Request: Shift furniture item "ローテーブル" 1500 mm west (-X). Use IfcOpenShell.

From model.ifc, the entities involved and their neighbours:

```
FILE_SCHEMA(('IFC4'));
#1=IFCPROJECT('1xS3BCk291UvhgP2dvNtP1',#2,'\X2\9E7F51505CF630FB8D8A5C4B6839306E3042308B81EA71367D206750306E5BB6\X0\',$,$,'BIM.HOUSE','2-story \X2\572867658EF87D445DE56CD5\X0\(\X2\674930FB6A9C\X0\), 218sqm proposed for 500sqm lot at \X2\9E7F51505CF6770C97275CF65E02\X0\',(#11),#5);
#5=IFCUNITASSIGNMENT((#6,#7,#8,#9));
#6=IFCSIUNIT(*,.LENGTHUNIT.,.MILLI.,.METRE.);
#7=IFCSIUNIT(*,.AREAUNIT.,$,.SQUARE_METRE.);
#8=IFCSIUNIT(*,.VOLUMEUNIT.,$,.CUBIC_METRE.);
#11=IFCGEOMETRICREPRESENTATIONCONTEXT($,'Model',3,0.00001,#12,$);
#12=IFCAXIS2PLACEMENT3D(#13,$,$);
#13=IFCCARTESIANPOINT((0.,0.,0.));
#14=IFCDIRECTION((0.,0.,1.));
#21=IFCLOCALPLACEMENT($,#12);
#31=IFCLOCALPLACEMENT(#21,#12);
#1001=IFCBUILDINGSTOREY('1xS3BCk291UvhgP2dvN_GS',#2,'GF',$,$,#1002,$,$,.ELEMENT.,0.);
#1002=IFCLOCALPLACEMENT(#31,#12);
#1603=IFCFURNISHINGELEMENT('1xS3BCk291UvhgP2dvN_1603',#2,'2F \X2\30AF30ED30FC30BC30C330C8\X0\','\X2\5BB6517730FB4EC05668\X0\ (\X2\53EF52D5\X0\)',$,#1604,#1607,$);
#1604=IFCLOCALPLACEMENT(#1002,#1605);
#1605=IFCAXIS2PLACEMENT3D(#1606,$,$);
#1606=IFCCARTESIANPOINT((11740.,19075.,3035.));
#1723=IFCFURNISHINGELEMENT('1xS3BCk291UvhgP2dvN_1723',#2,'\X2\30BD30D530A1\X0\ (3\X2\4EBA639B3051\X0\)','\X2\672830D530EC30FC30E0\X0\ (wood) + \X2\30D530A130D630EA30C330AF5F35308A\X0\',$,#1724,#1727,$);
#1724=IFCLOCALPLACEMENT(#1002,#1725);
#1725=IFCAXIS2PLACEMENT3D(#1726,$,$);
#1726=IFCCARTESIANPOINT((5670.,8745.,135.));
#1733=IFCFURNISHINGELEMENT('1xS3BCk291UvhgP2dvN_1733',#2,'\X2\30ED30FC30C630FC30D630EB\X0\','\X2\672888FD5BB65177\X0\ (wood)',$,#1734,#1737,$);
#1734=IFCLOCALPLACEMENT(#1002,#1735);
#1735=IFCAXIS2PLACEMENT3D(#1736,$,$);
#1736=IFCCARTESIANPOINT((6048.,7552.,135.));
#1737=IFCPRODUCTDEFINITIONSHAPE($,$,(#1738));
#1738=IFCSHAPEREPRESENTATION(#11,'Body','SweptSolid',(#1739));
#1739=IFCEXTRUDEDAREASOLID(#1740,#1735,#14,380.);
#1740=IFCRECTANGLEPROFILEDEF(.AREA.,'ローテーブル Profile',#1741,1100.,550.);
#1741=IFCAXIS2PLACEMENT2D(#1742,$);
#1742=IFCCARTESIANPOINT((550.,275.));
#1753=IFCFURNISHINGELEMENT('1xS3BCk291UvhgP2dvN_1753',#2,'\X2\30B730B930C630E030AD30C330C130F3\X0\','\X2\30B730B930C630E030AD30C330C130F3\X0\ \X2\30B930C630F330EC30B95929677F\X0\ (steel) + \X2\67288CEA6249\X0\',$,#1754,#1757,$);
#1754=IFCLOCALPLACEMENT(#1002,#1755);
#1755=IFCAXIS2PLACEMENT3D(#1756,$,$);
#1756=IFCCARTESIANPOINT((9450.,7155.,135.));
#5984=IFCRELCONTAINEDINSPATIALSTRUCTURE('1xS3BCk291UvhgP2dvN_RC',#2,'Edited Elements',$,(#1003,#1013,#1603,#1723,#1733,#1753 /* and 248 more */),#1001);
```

```python
import ifcopenshell
import ifcopenshell.api.geometry
import ifcopenshell.util.placement

model = ifcopenshell.open("model.ifc")

item = model.by_guid("1xS3BCk291UvhgP2dvN_1733")
matrix = ifcopenshell.util.placement.get_local_placement(item.ObjectPlacement)
matrix[0, 3] -= 1500.0
ifcopenshell.api.geometry.edit_object_placement(model, product=item, matrix=matrix, is_si=False)

print(ifcopenshell.util.placement.get_local_placement(item.ObjectPlacement).round(3) + 0.0)

model.write("model_updated.ifc")
```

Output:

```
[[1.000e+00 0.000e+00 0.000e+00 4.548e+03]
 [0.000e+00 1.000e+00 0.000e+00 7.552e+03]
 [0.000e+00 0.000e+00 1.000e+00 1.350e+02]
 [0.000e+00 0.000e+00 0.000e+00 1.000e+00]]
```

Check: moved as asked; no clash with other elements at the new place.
